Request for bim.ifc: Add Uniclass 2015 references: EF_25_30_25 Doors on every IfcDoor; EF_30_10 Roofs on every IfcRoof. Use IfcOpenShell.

First a look at what the model holds.

```python
import ifcopenshell

model = ifcopenshell.open("bim.ifc")
print(model.schema)
print("classifications:", [c.Name for c in model.by_type("IfcClassification")])
for ifc_class in ("IfcDoor", "IfcRoof", "IfcStair", "IfcWall", "IfcWindow"):
    print(ifc_class, len(model.by_type(ifc_class)))
```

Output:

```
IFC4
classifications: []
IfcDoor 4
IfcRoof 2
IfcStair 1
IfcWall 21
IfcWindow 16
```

```python
import ifcopenshell
import ifcopenshell.api.classification

model = ifcopenshell.open("bim.ifc")

system = ifcopenshell.api.classification.add_classification(model, classification="Uniclass 2015")

codes = {
    "IfcDoor": ("EF_25_30_25", "Doors"),
    "IfcRoof": ("EF_30_10", "Roofs"),
}
for ifc_class, (code, name) in codes.items():
    products = model.by_type(ifc_class)
    ifcopenshell.api.classification.add_reference(
        model, products=products, classification=system, identification=code, name=name
    )
    print(code, len(products))

model.write("bim_edited.ifc")
```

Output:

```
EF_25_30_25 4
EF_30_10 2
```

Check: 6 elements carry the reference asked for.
